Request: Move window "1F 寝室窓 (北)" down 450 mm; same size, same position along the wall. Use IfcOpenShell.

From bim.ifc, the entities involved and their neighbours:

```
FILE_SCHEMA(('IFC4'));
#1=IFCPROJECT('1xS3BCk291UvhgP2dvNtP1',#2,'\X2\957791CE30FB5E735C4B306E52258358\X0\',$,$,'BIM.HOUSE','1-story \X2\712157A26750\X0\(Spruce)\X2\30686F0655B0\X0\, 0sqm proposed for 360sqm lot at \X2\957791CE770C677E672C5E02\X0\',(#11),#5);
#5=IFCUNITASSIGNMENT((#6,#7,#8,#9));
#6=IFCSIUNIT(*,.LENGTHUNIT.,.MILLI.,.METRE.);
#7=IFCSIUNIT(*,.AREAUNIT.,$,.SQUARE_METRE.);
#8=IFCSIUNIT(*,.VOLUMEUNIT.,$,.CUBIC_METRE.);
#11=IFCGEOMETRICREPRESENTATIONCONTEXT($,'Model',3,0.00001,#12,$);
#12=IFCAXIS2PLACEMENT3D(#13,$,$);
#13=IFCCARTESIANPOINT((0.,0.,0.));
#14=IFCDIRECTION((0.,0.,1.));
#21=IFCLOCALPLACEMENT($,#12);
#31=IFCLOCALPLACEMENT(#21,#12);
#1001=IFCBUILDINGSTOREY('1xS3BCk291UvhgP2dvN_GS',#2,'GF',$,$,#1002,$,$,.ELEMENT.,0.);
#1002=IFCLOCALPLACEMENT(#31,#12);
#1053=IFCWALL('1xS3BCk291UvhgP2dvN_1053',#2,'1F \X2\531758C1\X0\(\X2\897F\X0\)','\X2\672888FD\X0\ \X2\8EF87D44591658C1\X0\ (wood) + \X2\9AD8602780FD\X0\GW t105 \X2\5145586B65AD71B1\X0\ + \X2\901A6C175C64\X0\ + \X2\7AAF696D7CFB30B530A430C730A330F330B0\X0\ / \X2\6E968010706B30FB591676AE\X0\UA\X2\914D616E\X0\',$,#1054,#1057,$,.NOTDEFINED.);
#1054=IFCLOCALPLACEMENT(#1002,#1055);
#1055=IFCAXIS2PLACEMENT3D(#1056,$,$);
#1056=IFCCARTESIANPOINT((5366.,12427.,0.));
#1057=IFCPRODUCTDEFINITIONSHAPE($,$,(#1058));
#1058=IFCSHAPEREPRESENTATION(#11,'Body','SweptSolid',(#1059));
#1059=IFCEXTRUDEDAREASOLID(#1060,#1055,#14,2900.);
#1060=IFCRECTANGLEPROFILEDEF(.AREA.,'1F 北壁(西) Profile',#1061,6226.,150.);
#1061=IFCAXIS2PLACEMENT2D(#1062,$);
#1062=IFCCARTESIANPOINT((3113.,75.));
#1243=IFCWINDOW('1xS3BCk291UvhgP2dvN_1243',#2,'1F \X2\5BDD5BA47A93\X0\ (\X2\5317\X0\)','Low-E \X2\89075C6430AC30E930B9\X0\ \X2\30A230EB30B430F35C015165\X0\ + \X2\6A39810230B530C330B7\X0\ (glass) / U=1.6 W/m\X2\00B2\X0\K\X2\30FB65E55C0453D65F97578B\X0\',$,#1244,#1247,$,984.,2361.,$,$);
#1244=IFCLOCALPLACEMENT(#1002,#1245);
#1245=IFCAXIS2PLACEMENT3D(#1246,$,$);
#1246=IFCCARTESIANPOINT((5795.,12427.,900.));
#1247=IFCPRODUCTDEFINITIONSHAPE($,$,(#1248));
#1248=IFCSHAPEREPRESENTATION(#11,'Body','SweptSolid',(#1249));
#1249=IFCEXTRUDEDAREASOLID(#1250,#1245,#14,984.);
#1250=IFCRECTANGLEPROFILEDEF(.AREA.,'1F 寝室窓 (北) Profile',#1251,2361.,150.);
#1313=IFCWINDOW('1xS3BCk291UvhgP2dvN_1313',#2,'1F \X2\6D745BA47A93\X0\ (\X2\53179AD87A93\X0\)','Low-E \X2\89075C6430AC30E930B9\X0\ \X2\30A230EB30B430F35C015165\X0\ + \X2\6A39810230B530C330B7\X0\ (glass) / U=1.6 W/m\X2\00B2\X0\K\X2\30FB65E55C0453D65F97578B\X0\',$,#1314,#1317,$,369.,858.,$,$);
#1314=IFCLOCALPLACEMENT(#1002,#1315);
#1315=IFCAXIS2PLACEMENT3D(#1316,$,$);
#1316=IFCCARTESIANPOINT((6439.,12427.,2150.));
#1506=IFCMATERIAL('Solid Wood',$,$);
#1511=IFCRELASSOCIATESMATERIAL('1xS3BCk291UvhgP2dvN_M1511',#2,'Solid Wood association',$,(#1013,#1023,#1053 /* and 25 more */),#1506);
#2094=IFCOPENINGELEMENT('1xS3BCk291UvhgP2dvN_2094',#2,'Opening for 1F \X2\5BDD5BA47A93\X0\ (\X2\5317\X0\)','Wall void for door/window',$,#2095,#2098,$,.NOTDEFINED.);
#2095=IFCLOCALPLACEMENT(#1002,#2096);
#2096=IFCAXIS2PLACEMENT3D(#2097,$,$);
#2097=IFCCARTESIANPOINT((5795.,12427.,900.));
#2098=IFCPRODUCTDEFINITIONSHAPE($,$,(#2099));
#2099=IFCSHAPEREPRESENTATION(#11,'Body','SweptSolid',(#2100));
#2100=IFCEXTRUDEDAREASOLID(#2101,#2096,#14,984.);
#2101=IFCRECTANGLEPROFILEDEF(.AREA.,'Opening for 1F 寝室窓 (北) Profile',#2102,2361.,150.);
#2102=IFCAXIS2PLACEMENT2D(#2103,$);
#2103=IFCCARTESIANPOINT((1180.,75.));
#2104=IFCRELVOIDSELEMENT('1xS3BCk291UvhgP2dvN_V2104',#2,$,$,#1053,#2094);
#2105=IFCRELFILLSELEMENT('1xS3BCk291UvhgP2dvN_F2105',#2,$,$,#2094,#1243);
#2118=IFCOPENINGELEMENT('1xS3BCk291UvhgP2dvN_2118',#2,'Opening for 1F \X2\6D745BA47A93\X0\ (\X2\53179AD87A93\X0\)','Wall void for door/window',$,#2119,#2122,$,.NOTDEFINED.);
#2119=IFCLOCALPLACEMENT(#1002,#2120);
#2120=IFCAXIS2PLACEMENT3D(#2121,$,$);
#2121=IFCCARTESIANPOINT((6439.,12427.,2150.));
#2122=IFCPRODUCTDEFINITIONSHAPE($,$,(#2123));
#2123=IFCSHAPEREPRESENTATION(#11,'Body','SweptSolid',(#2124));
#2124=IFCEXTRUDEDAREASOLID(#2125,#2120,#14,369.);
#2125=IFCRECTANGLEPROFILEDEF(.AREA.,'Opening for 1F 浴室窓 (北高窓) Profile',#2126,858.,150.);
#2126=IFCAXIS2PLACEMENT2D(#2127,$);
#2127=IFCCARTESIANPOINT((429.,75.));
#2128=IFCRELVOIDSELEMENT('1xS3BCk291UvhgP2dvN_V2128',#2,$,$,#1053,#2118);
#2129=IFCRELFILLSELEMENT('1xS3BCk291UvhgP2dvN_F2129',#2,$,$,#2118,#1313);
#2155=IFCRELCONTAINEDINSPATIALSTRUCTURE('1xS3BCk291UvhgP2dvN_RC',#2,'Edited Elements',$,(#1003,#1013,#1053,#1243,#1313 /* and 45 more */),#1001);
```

```python
import numpy as np
import ifcopenshell
import ifcopenshell.api.geometry
import ifcopenshell.util.placement
import ifcopenshell.util.unit

model = ifcopenshell.open("bim.ifc")
unit_scale = ifcopenshell.util.unit.calculate_unit_scale(model)

window = model.by_id(1243)
opening = window.FillsVoids[0].RelatingOpeningElement
dz = -450.0

shift = np.array([0.0, 0.0, dz])
# The window is not placed relative to its opening, so move both.
for product in (opening, window):
    matrix = ifcopenshell.util.placement.get_local_placement(product.ObjectPlacement)
    matrix[:3, 3] += shift
    ifcopenshell.api.geometry.edit_object_placement(model, product=product, matrix=matrix, is_si=False)

print(f"moved by {dz * unit_scale:+.3f} m")

model.write("bim-out.ifc")
```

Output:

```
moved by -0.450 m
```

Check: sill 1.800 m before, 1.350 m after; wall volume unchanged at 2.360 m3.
